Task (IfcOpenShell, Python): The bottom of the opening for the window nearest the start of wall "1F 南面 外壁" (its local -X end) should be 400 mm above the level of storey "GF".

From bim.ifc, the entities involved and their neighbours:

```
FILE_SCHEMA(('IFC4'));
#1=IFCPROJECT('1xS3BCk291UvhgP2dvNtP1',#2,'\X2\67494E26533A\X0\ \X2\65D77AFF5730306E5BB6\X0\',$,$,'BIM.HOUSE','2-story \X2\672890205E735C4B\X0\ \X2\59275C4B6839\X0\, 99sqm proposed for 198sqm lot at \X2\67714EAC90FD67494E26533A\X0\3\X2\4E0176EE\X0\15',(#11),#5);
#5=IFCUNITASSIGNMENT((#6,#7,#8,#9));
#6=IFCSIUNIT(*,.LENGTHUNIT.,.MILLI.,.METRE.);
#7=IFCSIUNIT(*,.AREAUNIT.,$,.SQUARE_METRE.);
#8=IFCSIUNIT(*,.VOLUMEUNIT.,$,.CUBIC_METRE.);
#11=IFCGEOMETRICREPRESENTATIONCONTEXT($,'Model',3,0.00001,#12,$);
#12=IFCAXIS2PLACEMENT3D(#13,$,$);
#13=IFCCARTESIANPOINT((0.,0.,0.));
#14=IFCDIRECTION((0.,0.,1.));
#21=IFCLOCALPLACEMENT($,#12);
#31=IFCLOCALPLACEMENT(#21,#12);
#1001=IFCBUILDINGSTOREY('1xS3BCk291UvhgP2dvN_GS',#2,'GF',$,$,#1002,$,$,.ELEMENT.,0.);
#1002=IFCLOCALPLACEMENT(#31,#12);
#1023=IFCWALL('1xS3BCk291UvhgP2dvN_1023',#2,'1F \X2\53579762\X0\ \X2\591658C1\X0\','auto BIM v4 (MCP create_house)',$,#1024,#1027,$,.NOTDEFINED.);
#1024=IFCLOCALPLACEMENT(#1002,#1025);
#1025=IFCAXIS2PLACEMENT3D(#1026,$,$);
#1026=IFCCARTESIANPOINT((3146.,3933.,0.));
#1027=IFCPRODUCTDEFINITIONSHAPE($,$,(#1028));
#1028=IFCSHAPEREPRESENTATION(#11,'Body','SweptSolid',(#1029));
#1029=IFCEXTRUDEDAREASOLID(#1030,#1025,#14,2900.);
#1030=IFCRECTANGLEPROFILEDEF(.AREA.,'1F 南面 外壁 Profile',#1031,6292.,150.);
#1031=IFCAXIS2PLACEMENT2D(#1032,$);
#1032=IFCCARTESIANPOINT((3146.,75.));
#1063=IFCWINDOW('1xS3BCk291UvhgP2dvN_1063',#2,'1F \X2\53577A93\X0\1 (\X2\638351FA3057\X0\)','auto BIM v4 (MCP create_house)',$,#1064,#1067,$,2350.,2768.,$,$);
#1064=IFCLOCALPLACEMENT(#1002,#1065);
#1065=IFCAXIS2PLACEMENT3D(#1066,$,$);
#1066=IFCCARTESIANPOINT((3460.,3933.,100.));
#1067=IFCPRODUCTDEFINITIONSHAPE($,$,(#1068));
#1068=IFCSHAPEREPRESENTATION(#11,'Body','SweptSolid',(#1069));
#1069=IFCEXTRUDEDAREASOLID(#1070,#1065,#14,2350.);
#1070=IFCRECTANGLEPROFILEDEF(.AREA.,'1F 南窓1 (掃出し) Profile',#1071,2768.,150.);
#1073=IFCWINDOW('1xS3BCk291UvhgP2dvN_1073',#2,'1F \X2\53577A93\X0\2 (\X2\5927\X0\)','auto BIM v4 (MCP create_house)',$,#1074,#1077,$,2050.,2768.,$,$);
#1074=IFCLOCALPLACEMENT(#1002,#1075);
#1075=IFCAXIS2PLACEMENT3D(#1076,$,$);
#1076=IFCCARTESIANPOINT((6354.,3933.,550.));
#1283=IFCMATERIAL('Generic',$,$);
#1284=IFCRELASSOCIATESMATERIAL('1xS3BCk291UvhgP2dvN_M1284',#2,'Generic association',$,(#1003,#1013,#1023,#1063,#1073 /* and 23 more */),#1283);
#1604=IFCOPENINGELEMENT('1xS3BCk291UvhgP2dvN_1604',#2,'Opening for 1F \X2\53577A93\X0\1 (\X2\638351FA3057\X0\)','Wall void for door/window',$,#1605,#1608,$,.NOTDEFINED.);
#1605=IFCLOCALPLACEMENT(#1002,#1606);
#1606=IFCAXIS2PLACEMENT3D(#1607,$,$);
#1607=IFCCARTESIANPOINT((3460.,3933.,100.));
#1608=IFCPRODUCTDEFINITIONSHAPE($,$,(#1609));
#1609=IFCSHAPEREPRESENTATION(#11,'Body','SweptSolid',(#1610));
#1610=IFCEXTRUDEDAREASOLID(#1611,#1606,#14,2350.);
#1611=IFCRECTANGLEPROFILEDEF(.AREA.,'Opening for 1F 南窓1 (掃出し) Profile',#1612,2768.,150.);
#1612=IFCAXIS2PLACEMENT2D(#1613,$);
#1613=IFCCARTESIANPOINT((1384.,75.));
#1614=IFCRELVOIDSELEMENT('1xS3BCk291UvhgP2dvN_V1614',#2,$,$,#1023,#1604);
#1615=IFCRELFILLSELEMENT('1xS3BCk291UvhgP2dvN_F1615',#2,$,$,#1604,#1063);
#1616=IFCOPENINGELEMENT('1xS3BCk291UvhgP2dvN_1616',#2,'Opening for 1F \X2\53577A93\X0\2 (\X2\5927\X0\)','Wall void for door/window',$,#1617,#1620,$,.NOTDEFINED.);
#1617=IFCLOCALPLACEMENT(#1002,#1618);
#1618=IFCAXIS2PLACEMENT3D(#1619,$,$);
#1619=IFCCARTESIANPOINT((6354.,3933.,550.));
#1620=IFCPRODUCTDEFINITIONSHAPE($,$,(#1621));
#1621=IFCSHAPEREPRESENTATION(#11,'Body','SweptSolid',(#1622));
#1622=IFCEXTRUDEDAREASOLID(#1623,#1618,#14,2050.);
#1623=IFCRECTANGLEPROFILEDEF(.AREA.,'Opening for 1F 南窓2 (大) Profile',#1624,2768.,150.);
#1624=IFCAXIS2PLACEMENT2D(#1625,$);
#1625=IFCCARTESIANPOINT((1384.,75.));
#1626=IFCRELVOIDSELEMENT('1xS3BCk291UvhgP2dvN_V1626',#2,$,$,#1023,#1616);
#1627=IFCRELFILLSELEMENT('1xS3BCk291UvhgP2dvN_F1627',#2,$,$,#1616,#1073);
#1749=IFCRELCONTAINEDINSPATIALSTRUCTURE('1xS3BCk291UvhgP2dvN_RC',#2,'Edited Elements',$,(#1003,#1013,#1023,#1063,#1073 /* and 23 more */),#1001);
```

```python
import numpy as np
import ifcopenshell
import ifcopenshell.api.geometry
import ifcopenshell.geom
import ifcopenshell.util.element
import ifcopenshell.util.placement
import ifcopenshell.util.shape
import ifcopenshell.util.unit

model = ifcopenshell.open("bim.ifc")
unit_scale = ifcopenshell.util.unit.calculate_unit_scale(model)

window = model.by_guid("1xS3BCk291UvhgP2dvN_1063")
opening = window.FillsVoids[0].RelatingOpeningElement
storey = ifcopenshell.util.element.get_container(window, ifc_class="IfcBuildingStorey")
level = ifcopenshell.util.placement.get_local_placement(storey.ObjectPlacement)[2, 3]

# The opening's origin need not be at the sill, so measure its lowest point.
shape = ifcopenshell.geom.create_shape(ifcopenshell.geom.settings(), opening)
bottom = ifcopenshell.util.shape.get_shape_bottom_elevation(shape, shape.geometry) / unit_scale
dz = level + 0.4 / unit_scale - bottom

shift = np.array([0.0, 0.0, dz])
# The window is not placed relative to its opening, so move both.
for product in (opening, window):
    matrix = ifcopenshell.util.placement.get_local_placement(product.ObjectPlacement)
    matrix[:3, 3] += shift
    ifcopenshell.api.geometry.edit_object_placement(model, product=product, matrix=matrix, is_si=False)

print(f"moved by {dz * unit_scale:+.3f} m")

model.write("bim_updated.ifc")
```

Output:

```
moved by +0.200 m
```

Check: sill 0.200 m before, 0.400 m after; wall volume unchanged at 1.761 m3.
